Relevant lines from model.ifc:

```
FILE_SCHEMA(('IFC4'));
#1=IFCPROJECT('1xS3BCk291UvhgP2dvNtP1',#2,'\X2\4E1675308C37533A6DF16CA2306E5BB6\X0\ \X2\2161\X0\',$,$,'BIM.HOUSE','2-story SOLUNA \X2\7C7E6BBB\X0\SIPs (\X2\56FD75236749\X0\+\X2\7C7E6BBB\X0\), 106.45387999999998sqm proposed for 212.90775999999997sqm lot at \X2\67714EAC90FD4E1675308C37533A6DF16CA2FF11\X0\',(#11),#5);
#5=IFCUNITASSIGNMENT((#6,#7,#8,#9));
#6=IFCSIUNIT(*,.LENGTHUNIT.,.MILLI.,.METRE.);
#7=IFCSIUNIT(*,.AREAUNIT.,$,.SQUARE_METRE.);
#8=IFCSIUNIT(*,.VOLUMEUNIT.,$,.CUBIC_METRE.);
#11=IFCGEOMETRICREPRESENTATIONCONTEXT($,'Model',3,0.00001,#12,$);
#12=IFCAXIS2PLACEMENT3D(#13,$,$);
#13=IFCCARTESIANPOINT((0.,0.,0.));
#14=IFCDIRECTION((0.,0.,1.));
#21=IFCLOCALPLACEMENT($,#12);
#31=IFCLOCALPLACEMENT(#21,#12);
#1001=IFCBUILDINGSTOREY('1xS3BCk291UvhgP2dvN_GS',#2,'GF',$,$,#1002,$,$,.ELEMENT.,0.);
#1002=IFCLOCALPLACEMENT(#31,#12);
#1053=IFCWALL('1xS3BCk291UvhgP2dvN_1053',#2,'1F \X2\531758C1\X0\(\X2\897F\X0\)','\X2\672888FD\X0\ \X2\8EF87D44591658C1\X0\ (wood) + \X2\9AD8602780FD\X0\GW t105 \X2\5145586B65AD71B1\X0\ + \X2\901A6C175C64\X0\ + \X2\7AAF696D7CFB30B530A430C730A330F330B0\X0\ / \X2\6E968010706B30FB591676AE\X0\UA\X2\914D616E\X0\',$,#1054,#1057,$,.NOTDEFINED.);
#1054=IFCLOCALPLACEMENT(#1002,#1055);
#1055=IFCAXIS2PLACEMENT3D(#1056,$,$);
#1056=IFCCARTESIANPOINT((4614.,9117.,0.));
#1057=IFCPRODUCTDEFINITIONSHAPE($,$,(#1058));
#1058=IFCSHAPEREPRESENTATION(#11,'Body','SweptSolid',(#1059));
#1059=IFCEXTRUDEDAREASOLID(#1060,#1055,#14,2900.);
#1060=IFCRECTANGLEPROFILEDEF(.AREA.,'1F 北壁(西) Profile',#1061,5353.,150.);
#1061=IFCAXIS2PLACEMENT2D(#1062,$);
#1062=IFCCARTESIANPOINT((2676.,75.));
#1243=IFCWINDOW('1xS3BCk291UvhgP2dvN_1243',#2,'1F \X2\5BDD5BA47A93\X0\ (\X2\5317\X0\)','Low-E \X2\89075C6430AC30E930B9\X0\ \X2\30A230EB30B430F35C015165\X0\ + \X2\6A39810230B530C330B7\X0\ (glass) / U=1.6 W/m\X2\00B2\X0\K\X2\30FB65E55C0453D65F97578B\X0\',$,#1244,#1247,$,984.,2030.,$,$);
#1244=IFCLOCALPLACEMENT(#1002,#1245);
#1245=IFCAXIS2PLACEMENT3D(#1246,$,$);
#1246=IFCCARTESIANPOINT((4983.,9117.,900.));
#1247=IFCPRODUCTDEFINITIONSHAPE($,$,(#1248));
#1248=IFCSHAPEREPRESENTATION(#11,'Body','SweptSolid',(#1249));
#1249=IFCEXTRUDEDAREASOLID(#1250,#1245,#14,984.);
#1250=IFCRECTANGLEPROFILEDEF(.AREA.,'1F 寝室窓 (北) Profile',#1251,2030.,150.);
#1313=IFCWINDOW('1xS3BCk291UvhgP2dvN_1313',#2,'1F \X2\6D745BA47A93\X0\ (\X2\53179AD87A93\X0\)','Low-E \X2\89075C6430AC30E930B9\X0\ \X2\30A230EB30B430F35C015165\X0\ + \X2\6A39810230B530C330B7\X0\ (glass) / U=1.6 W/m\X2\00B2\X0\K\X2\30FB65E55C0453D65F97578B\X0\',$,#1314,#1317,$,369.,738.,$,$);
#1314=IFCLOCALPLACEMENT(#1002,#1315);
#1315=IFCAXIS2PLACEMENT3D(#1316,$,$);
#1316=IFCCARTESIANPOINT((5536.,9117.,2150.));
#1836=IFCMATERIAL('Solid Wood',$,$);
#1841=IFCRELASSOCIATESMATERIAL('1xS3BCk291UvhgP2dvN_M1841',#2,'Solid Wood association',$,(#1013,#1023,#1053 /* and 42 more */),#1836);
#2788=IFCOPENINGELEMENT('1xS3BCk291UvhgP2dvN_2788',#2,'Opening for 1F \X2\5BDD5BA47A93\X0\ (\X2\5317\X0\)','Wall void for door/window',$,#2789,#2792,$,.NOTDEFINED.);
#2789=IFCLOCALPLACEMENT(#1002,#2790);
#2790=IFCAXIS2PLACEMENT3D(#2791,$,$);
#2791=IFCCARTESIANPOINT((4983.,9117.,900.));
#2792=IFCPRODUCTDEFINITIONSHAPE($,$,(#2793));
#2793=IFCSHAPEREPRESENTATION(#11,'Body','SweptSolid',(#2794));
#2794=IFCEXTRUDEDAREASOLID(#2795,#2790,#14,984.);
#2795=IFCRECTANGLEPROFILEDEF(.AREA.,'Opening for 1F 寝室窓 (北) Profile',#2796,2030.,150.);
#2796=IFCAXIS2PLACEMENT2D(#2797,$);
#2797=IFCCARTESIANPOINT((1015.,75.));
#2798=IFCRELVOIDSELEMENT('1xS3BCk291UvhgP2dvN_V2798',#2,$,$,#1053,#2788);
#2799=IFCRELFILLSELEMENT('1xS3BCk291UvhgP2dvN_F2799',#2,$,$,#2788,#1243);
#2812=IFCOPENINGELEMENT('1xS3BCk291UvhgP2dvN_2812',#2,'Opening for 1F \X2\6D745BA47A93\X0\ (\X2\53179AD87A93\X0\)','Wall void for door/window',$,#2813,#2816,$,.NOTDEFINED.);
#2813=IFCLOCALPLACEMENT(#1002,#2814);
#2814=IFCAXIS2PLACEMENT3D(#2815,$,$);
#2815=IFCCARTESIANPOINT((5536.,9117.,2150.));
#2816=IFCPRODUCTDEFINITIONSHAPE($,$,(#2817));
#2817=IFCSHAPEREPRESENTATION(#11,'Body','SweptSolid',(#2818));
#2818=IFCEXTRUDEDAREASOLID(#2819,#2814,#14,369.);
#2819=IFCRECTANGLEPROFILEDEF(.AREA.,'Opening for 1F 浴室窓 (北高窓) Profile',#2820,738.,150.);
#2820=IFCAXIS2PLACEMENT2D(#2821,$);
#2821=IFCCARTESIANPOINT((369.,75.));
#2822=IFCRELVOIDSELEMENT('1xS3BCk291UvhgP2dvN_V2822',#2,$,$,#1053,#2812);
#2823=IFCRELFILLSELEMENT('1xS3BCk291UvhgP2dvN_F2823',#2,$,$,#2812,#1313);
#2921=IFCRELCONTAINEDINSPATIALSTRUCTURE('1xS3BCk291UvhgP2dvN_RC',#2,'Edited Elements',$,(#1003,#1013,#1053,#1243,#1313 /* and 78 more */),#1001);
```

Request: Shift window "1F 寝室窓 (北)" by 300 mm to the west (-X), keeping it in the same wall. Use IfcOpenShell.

```python
import ifcopenshell
import ifcopenshell.api.geometry
import ifcopenshell.util.placement

model = ifcopenshell.open("model.ifc")

window = model.by_id(1243)
opening = window.FillsVoids[0].RelatingOpeningElement
wall = opening.VoidsElements[0].RelatingBuildingElement

wall_matrix = ifcopenshell.util.placement.get_local_placement(wall.ObjectPlacement)
shift = wall_matrix[:3, 0] * -300.0
before = ifcopenshell.util.placement.get_local_placement(window.ObjectPlacement)[:3, 3].copy()

# The window is not placed relative to its opening, so move both.
for product in (opening, window):
    matrix = ifcopenshell.util.placement.get_local_placement(product.ObjectPlacement)
    matrix[:3, 3] += shift
    ifcopenshell.api.geometry.edit_object_placement(model, product=product, matrix=matrix, is_si=False)

after = ifcopenshell.util.placement.get_local_placement(window.ObjectPlacement)[:3, 3]
print("window moved by", (after - before).round(3) + 0.0)

model.write("model_v2.ifc")
```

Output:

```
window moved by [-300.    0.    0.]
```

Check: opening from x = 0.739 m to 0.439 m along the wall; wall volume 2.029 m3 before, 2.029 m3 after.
